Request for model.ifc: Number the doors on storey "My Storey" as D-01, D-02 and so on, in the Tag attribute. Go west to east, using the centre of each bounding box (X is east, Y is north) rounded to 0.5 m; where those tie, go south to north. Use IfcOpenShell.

First a look at what the model holds.

```python
import ifcopenshell
import ifcopenshell.util.element
import ifcopenshell.util.placement

model = ifcopenshell.open("model.ifc")
print(model.schema)
storey = next(s for s in model.by_type("IfcBuildingStorey") if s.Name == "My Storey")
doors = [e for e in ifcopenshell.util.element.get_decomposition(storey) if e.is_a("IfcDoor")]
for e in sorted(doors, key=lambda e: e.id()):
    origin = ifcopenshell.util.placement.get_local_placement(e.ObjectPlacement)[:3, 3]
    print(e.id(), e.Tag, e.Name, origin.round(2) + 0.0, sep=" | ")
```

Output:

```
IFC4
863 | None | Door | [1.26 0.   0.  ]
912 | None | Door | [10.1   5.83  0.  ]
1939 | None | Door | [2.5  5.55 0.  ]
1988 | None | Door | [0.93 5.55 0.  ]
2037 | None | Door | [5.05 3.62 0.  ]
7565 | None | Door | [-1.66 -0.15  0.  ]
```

```python
import ifcopenshell
import ifcopenshell.geom
import ifcopenshell.util.element
import ifcopenshell.util.shape

model = ifcopenshell.open("model.ifc")
settings = ifcopenshell.geom.settings()
settings.set("use-world-coords", True)


def centre(element):
    shape = ifcopenshell.geom.create_shape(settings, element)
    return ifcopenshell.util.shape.get_bbox_centroid(shape.geometry)


storey = next(s for s in model.by_type("IfcBuildingStorey") if s.Name == "My Storey")
doors = [e for e in ifcopenshell.util.element.get_decomposition(storey) if e.is_a("IfcDoor")]

# Insertion points can sit at a corner or the storey origin, so sort by the geometry (in metres).
centres = {e: centre(e) for e in doors}
doors.sort(key=lambda e: (round(centres[e][0] / 0.5), centres[e][1]))

for i, e in enumerate(doors, start=1):
    number = f"D-{i:02d}"
    e.Tag = number
    print(e.id(), number)

model.write("model_rev.ifc")
```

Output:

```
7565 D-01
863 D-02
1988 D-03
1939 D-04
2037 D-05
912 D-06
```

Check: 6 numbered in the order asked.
